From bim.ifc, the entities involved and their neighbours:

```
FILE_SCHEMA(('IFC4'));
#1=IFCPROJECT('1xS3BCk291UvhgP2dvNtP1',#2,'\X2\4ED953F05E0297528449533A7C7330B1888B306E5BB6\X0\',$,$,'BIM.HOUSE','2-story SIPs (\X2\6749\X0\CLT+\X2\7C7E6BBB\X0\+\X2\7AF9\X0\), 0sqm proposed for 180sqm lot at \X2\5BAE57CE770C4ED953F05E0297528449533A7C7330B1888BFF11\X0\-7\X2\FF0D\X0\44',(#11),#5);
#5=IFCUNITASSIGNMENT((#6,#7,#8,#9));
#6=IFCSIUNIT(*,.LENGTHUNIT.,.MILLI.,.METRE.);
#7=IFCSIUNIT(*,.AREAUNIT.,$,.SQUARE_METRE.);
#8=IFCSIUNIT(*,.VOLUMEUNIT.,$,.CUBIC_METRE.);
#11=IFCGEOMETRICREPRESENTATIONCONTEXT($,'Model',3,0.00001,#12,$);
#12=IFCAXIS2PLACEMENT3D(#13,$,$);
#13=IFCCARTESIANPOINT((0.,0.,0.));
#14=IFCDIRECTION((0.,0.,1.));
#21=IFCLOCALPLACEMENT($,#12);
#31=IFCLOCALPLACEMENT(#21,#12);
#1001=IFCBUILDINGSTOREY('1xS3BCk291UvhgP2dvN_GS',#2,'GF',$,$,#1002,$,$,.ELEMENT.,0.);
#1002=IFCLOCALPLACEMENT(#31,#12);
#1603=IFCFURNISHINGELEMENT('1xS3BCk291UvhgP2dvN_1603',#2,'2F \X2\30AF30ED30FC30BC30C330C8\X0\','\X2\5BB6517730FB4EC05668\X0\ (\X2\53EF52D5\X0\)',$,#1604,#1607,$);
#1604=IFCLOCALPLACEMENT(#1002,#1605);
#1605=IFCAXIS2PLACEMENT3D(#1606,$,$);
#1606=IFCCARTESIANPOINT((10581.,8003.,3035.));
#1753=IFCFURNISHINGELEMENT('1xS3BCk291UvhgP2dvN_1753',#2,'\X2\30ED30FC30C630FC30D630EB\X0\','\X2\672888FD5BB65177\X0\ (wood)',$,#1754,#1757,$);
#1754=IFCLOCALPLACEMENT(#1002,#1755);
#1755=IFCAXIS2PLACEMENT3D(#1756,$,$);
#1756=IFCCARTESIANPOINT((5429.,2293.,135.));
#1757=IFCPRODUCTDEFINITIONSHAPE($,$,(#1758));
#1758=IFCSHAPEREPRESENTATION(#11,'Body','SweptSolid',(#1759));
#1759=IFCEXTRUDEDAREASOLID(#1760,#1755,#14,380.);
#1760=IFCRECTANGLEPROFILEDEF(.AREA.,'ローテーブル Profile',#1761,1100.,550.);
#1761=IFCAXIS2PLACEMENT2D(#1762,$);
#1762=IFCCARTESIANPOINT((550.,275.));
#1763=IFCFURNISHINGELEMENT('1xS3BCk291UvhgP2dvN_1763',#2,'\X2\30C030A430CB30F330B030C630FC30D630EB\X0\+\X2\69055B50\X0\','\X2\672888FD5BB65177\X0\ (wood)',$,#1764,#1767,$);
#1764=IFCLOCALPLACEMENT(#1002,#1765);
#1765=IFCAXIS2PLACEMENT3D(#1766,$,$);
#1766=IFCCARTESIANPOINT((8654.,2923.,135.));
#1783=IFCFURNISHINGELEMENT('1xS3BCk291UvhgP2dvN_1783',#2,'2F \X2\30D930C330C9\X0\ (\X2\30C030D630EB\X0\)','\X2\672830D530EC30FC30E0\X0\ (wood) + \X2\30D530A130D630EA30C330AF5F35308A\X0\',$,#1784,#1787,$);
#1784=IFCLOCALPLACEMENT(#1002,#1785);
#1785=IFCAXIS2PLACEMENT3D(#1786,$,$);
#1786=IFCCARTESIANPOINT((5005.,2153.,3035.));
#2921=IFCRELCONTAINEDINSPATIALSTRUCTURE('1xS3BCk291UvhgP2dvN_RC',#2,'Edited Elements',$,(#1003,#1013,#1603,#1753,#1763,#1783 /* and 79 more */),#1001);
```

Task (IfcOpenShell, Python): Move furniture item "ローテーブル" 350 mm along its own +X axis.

```python
import ifcopenshell
import ifcopenshell.api.geometry
import ifcopenshell.util.placement

model = ifcopenshell.open("bim.ifc")

item = model.by_guid("1xS3BCk291UvhgP2dvN_1753")
matrix = ifcopenshell.util.placement.get_local_placement(item.ObjectPlacement)
matrix[:3, 3] += matrix[:3, 0] * 350.0
ifcopenshell.api.geometry.edit_object_placement(model, product=item, matrix=matrix, is_si=False)

print(ifcopenshell.util.placement.get_local_placement(item.ObjectPlacement).round(3) + 0.0)

model.write("bim-out.ifc")
```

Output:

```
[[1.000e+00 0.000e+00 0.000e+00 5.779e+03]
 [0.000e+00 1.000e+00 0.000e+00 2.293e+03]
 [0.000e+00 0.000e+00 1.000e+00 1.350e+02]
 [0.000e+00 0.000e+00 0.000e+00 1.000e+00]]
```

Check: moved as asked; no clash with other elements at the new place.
